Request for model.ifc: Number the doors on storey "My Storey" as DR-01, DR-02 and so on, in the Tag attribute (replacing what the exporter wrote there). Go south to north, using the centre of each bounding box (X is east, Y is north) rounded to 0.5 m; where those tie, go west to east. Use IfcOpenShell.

First a look at what the model holds.

```python
import ifcopenshell
import ifcopenshell.util.element
import ifcopenshell.util.placement

model = ifcopenshell.open("model.ifc")
print(model.schema)
storey = next(s for s in model.by_type("IfcBuildingStorey") if s.Name == "My Storey")
doors = [e for e in ifcopenshell.util.element.get_decomposition(storey) if e.is_a("IfcDoor")]
for e in sorted(doors, key=lambda e: e.id()):
    origin = ifcopenshell.util.placement.get_local_placement(e.ObjectPlacement)[:3, 3]
    print(e.id(), e.Tag, e.Name, origin.round(2) + 0.0, sep=" | ")
```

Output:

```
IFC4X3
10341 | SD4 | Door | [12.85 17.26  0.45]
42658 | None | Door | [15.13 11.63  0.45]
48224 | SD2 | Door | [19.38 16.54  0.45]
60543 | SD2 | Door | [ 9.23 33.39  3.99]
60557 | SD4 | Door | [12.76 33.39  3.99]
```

```python
import ifcopenshell
import ifcopenshell.geom
import ifcopenshell.util.element
import ifcopenshell.util.shape

model = ifcopenshell.open("model.ifc")
settings = ifcopenshell.geom.settings()
settings.set("use-world-coords", True)


def centre(element):
    shape = ifcopenshell.geom.create_shape(settings, element)
    return ifcopenshell.util.shape.get_bbox_centroid(shape.geometry)


storey = next(s for s in model.by_type("IfcBuildingStorey") if s.Name == "My Storey")
doors = [e for e in ifcopenshell.util.element.get_decomposition(storey) if e.is_a("IfcDoor")]

# Insertion points can sit at a corner or the storey origin, so sort by the geometry (in metres).
centres = {e: centre(e) for e in doors}
doors.sort(key=lambda e: (round(centres[e][1] / 0.5), centres[e][0]))

for i, e in enumerate(doors, start=1):
    number = f"DR-{i:02d}"
    e.Tag = number
    print(e.id(), number)

model.write("model_rev.ifc")
```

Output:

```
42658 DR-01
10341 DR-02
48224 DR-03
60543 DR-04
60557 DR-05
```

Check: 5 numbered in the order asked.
